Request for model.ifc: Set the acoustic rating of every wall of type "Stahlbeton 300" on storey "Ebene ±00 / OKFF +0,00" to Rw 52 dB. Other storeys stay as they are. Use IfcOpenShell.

First a look at what the model holds.

```python
import ifcopenshell
import ifcopenshell.util.element

model = ifcopenshell.open("model.ifc")
print(model.schema)
storey = next(s for s in model.by_type("IfcBuildingStorey") if s.Name == "Ebene ±00 / OKFF +0,00")
walls = [e for e in ifcopenshell.util.element.get_decomposition(storey) if e.is_a("IfcWall")]
seen = {}
for e in walls:
    element_type = ifcopenshell.util.element.get_type(e)
    key = (element_type.Name if element_type != e and element_type else None, ifcopenshell.util.element.get_pset(e, "Pset_WallCommon", "AcousticRating"))
    seen[key] = seen.get(key, 0) + 1
for (name, value), count in sorted(seen.items(), key=str):
    print(count, "x", name, "|", value)
```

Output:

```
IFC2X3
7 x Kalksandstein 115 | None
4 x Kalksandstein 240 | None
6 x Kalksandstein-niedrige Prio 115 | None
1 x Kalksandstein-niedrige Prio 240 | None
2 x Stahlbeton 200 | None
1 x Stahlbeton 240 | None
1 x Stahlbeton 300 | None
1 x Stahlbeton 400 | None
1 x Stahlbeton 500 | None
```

```python
import ifcopenshell
import ifcopenshell.api.pset
import ifcopenshell.util.element

model = ifcopenshell.open("model.ifc")

storey = next(s for s in model.by_type("IfcBuildingStorey") if s.Name == "Ebene ±00 / OKFF +0,00")
walls = [e for e in ifcopenshell.util.element.get_decomposition(storey) if e.is_a("IfcWall")]

count = 0
for e in walls:
    element_type = ifcopenshell.util.element.get_type(e)
    if element_type in (None, e) or element_type.Name != "Stahlbeton 300":
        continue
    # add_pset returns the element's existing set when there is one.
    pset = ifcopenshell.api.pset.add_pset(model, product=e, name="Pset_WallCommon")
    ifcopenshell.api.pset.edit_pset(model, pset=pset, properties={"AcousticRating": "Rw 52 dB"})
    count += 1

print(count, "walls updated")

model.write("model-out.ifc")
```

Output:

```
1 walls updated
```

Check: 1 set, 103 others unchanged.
